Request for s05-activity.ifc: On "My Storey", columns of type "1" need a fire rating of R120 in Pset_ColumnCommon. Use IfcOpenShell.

First a look at what the model holds.

```python
import ifcopenshell
import ifcopenshell.util.element

model = ifcopenshell.open("s05-activity.ifc")
print(model.schema)
storey = next(s for s in model.by_type("IfcBuildingStorey") if s.Name == "My Storey")
columns = [e for e in ifcopenshell.util.element.get_decomposition(storey) if e.is_a("IfcColumn")]
seen = {}
for e in columns:
    element_type = ifcopenshell.util.element.get_type(e)
    key = (element_type.Name if element_type != e and element_type else None, ifcopenshell.util.element.get_pset(e, "Pset_ColumnCommon", "FireRating"))
    seen[key] = seen.get(key, 0) + 1
for (name, value), count in sorted(seen.items(), key=str):
    print(count, "x", name, "|", value)
```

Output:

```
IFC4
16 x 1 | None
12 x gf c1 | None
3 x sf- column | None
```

```python
import ifcopenshell
import ifcopenshell.api.pset
import ifcopenshell.util.element

model = ifcopenshell.open("s05-activity.ifc")

storey = next(s for s in model.by_type("IfcBuildingStorey") if s.Name == "My Storey")
columns = [e for e in ifcopenshell.util.element.get_decomposition(storey) if e.is_a("IfcColumn")]

count = 0
for e in columns:
    element_type = ifcopenshell.util.element.get_type(e)
    if element_type in (None, e) or element_type.Name != "1":
        continue
    # add_pset returns the element's existing set when there is one.
    pset = ifcopenshell.api.pset.add_pset(model, product=e, name="Pset_ColumnCommon")
    ifcopenshell.api.pset.edit_pset(model, pset=pset, properties={"FireRating": "R120"})
    count += 1

print(count, "columns updated")

model.write("s05-activity_edited.ifc")
```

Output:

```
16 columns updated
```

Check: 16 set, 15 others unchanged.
